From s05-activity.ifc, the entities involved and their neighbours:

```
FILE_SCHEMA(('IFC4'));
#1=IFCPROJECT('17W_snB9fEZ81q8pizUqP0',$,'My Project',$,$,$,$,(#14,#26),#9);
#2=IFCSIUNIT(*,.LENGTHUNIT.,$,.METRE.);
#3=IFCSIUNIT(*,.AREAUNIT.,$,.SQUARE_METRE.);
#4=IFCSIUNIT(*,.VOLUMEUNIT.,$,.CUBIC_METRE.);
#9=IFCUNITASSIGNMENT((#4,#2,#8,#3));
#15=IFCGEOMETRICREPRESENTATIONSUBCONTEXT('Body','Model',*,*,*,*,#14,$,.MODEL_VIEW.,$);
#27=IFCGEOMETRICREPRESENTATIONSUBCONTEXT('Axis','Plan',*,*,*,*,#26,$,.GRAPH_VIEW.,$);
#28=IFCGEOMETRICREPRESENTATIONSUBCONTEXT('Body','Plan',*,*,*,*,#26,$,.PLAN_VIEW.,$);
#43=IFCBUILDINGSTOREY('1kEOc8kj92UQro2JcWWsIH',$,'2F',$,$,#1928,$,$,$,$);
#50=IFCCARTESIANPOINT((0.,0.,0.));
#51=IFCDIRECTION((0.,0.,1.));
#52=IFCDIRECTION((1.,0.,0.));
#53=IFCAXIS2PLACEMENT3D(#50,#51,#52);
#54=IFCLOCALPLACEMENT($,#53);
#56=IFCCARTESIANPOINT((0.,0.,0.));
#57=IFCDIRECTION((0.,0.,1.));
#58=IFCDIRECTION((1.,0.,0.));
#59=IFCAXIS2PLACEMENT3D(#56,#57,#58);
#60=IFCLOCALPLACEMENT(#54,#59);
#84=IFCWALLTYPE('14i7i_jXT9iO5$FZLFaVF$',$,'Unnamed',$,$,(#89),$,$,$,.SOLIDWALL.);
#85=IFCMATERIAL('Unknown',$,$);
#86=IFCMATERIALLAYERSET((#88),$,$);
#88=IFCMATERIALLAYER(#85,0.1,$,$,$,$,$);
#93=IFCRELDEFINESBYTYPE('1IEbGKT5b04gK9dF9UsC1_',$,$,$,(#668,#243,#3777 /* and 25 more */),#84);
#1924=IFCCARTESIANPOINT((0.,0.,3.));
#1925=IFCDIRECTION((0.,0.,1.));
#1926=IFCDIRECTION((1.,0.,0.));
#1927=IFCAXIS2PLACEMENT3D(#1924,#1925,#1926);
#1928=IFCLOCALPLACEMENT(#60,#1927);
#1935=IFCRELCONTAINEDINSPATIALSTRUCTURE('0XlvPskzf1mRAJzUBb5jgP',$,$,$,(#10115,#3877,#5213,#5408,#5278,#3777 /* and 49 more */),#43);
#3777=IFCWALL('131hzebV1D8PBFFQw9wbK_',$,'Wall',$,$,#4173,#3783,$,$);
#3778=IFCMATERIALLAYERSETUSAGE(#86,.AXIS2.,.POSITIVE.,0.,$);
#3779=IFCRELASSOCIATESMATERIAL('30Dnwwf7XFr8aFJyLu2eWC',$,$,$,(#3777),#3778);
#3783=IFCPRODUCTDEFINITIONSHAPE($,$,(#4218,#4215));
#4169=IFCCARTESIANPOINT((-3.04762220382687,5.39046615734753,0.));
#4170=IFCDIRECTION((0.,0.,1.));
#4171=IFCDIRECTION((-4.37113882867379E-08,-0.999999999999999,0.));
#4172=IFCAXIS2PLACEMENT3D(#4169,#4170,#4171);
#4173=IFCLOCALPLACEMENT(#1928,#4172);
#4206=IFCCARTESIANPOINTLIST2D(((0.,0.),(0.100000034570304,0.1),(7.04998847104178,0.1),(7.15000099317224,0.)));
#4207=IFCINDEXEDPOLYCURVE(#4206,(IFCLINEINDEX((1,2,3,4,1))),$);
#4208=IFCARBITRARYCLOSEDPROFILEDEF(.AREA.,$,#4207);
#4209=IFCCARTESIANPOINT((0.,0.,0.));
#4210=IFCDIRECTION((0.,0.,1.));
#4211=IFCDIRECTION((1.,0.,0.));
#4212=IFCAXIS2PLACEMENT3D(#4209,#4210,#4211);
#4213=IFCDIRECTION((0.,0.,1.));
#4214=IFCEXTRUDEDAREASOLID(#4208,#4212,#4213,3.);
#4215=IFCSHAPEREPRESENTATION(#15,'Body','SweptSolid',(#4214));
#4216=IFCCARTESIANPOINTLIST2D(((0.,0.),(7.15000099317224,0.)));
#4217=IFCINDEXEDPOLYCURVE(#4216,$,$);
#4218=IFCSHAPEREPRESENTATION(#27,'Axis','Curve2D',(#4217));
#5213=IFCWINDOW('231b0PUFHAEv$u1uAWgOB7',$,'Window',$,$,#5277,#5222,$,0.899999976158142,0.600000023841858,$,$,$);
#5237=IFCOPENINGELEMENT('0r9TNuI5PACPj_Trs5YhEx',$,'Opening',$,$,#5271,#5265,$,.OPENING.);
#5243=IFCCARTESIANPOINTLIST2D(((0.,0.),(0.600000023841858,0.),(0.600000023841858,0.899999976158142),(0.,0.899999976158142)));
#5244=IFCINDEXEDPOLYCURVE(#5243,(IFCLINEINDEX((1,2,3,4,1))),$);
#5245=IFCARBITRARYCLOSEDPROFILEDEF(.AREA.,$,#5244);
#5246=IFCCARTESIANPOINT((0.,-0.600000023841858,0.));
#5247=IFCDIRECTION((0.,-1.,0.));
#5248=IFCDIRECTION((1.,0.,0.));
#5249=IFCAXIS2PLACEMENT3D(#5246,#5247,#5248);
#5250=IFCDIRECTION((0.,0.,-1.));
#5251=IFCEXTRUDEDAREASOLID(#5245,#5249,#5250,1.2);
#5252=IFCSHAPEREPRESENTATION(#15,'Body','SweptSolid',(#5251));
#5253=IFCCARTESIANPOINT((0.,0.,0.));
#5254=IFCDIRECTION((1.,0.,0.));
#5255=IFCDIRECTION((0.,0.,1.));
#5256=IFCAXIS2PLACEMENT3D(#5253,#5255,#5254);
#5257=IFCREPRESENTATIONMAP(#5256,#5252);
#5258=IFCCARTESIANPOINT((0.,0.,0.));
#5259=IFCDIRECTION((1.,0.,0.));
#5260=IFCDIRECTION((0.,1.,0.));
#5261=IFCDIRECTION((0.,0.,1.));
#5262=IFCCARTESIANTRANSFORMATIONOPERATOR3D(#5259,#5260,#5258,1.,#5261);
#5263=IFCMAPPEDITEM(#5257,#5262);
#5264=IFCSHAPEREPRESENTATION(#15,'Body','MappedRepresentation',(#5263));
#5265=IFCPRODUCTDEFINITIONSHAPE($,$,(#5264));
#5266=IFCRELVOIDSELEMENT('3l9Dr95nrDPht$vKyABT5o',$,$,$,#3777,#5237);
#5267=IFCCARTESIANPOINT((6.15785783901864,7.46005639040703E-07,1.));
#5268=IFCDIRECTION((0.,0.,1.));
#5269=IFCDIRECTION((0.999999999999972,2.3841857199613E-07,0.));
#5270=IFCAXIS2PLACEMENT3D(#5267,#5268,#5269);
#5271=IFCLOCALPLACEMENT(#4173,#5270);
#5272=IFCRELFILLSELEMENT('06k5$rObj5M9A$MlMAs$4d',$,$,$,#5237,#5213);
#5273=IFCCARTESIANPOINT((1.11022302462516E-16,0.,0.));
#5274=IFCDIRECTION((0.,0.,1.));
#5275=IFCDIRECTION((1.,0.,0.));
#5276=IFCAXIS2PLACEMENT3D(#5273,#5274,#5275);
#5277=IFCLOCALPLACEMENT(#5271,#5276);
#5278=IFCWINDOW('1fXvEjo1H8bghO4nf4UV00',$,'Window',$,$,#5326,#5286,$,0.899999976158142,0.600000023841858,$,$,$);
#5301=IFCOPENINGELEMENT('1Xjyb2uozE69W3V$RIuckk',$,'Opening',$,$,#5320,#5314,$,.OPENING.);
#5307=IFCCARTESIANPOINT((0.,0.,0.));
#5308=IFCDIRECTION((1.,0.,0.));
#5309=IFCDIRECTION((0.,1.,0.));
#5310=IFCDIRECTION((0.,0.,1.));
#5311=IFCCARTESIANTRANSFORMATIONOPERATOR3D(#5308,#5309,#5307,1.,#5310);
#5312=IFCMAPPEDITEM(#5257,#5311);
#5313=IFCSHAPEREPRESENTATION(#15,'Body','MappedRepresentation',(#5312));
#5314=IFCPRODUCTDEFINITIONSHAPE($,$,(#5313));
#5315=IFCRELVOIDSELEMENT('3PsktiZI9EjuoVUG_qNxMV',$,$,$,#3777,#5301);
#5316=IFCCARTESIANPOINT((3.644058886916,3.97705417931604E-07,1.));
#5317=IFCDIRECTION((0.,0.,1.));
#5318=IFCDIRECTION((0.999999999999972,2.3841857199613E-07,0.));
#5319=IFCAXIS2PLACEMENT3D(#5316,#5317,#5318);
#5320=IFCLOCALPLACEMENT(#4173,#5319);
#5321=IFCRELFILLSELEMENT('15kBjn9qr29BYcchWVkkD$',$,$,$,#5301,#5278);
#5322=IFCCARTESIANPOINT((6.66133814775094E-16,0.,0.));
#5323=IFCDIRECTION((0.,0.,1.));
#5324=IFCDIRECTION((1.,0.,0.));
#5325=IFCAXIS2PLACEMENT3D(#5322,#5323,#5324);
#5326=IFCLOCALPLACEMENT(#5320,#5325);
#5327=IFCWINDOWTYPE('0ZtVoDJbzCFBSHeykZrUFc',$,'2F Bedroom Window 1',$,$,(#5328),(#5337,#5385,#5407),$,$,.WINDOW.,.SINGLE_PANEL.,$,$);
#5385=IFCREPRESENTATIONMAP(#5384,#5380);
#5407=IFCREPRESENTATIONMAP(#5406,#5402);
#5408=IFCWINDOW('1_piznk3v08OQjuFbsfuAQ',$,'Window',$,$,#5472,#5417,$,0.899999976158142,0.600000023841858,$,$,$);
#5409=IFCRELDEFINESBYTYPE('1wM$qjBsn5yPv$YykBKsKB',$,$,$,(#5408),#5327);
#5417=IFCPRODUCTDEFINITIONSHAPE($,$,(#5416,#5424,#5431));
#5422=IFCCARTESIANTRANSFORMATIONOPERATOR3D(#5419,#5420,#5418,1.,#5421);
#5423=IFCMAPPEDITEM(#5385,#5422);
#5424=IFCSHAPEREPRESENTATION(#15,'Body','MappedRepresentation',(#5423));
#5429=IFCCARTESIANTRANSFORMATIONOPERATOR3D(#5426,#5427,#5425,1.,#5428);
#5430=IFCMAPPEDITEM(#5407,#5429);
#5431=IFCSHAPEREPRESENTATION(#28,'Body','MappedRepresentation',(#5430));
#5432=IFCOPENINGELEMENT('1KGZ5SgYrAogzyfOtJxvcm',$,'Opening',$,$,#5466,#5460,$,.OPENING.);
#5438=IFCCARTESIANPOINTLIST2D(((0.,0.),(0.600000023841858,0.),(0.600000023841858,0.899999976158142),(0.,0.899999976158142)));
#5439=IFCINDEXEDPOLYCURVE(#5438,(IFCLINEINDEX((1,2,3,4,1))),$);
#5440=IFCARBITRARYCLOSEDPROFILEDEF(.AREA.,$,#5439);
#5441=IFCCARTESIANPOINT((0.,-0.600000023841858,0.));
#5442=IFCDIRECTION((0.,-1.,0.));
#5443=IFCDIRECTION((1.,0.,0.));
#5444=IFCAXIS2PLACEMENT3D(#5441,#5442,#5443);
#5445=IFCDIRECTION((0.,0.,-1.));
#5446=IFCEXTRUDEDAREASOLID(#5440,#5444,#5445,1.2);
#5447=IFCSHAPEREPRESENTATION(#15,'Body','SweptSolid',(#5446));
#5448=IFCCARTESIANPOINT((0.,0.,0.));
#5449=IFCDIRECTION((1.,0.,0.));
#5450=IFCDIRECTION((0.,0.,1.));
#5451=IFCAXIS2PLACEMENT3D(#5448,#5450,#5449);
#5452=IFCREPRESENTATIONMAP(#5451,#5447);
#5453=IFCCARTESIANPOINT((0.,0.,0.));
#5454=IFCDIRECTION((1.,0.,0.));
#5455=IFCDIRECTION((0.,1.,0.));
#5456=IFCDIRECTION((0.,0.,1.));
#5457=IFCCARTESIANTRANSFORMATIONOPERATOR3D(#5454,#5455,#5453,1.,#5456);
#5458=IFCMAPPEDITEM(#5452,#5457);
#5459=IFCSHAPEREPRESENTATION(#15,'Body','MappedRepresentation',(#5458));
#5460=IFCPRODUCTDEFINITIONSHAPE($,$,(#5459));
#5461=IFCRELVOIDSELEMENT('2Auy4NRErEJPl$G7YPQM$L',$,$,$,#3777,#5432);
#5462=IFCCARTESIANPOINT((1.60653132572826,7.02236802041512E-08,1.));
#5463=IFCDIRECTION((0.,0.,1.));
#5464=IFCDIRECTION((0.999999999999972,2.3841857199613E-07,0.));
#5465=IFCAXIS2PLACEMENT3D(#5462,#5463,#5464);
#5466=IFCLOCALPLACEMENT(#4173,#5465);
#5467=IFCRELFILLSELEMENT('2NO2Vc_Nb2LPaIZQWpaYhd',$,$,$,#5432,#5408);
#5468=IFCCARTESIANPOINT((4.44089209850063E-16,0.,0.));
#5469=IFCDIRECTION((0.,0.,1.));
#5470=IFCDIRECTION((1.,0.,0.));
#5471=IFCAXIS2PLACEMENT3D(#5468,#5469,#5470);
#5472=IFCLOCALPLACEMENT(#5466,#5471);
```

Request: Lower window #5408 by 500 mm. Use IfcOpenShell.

```python
import numpy as np
import ifcopenshell
import ifcopenshell.api.geometry
import ifcopenshell.util.placement
import ifcopenshell.util.unit

model = ifcopenshell.open("s05-activity.ifc")
unit_scale = ifcopenshell.util.unit.calculate_unit_scale(model)

window = model.by_guid("1_piznk3v08OQjuFbsfuAQ")
opening = window.FillsVoids[0].RelatingOpeningElement
dz = -0.5 / unit_scale

shift = np.array([0.0, 0.0, dz])
# The window is placed relative to its opening, so it follows when the opening moves.
matrix = ifcopenshell.util.placement.get_local_placement(opening.ObjectPlacement)
matrix[:3, 3] += shift
ifcopenshell.api.geometry.edit_object_placement(
    model, product=opening, matrix=matrix, is_si=False, should_transform_children=True
)

print(f"moved by {dz * unit_scale:+.3f} m")

model.write("s05-activity_updated.ifc")
```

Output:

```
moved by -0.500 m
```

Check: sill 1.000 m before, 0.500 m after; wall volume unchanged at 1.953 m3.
